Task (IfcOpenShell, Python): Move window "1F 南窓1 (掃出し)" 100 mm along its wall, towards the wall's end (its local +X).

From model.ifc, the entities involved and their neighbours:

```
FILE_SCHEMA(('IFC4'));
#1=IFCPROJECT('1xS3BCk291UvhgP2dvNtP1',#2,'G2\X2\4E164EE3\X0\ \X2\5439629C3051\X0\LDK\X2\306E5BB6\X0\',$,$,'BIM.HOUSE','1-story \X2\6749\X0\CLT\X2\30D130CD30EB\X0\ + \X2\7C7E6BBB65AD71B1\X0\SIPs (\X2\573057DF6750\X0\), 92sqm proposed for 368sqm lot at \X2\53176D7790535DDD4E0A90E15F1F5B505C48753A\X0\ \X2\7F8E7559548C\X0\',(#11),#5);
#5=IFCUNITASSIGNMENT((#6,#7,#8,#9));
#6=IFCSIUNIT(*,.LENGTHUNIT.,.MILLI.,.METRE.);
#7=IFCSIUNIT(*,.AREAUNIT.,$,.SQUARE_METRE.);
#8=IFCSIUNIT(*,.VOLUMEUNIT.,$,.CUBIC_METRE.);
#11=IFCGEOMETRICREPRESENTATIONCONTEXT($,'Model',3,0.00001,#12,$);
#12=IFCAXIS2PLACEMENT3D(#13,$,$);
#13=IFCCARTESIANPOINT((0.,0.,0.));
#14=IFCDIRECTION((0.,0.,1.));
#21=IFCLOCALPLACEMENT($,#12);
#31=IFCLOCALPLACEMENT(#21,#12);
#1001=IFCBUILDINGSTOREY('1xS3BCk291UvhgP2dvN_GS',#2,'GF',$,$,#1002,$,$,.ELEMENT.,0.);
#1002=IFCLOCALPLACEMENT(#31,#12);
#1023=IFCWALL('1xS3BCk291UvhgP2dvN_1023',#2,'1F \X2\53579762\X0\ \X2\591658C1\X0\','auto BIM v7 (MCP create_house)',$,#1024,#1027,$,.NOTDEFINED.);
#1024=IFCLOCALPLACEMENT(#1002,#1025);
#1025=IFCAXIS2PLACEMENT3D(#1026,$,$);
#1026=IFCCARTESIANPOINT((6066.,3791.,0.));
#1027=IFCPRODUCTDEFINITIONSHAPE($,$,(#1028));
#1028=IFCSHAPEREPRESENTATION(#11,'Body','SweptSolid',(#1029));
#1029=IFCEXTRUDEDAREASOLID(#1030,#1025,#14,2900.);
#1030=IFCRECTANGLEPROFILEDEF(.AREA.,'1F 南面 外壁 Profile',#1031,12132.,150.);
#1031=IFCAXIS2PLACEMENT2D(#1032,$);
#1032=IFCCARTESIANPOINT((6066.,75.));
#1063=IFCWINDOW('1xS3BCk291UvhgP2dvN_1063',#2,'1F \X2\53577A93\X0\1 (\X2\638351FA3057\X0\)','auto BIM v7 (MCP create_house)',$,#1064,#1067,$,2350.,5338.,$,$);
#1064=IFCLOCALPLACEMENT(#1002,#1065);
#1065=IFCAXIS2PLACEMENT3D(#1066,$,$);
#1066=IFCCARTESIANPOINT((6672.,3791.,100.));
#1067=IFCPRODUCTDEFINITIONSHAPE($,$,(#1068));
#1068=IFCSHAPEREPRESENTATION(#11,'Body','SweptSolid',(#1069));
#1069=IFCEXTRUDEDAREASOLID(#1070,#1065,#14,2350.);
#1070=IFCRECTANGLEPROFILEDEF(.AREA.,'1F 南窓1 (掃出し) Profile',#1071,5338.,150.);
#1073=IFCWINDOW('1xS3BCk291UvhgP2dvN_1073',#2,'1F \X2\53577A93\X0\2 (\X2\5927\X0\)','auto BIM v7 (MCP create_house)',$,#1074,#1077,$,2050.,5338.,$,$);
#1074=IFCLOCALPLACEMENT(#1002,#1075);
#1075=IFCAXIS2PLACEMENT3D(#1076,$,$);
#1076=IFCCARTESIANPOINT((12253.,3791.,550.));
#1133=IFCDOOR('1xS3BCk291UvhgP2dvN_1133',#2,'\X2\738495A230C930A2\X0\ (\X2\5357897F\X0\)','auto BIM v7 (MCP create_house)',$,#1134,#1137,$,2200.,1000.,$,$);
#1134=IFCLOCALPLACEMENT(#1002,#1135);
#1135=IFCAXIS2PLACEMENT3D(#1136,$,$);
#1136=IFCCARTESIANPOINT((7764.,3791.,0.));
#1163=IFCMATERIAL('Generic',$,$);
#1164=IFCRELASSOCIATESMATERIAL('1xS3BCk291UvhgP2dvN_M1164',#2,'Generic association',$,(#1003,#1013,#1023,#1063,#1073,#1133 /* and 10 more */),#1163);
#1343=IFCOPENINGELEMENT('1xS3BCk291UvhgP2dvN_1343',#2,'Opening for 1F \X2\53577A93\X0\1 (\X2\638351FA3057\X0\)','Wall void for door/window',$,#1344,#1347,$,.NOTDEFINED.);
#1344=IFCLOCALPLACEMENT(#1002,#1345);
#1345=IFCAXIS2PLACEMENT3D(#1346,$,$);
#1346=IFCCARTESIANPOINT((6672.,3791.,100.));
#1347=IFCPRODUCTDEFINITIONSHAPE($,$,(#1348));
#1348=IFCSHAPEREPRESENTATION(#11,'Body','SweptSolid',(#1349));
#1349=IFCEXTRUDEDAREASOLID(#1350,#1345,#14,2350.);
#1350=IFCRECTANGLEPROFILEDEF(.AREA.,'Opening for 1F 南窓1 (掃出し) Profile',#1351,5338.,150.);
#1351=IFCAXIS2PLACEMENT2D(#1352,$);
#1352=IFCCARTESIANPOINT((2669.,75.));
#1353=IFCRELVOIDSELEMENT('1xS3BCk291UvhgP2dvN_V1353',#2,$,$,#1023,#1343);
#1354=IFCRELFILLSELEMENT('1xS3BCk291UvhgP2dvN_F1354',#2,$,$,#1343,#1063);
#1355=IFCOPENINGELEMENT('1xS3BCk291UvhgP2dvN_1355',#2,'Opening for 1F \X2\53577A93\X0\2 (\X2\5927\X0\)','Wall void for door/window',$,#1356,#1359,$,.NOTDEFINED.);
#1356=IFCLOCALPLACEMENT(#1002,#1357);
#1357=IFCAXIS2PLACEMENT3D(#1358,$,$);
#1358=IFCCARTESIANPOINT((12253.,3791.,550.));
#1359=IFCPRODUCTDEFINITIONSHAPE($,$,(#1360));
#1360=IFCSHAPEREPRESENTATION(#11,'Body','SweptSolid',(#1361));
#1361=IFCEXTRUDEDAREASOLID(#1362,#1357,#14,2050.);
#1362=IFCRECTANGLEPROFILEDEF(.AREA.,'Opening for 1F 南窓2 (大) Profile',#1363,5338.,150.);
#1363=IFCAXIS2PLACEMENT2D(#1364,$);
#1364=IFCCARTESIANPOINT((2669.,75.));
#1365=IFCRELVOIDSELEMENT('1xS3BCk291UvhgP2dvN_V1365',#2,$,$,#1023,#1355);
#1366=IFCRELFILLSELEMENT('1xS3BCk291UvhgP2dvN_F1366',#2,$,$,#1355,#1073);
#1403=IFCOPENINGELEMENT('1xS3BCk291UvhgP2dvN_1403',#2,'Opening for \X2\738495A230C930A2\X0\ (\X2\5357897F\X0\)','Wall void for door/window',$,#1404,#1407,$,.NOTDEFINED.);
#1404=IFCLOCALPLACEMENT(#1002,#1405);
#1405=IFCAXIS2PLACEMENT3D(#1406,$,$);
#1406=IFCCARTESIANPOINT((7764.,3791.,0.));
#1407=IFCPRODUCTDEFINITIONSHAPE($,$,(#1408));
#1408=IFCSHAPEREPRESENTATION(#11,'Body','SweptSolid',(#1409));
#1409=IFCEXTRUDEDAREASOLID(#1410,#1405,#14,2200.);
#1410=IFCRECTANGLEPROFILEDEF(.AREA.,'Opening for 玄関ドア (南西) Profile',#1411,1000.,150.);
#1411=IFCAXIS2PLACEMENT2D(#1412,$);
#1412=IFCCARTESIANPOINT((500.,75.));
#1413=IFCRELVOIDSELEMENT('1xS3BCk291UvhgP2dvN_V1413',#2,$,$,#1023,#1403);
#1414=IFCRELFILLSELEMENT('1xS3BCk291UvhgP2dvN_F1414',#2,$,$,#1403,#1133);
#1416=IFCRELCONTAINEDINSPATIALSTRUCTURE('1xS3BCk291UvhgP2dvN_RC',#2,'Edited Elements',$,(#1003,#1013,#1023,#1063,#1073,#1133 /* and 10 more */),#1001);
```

```python
import ifcopenshell
import ifcopenshell.api.geometry
import ifcopenshell.util.placement
import ifcopenshell.util.unit

model = ifcopenshell.open("model.ifc")
unit_scale = ifcopenshell.util.unit.calculate_unit_scale(model)

window = model.by_id(1063)
opening = window.FillsVoids[0].RelatingOpeningElement
wall = opening.VoidsElements[0].RelatingBuildingElement

wall_matrix = ifcopenshell.util.placement.get_local_placement(wall.ObjectPlacement)
shift = wall_matrix[:3, 0] * 0.1 / unit_scale
before = ifcopenshell.util.placement.get_local_placement(window.ObjectPlacement)[:3, 3].copy()

# The window is not placed relative to its opening, so move both.
for product in (opening, window):
    matrix = ifcopenshell.util.placement.get_local_placement(product.ObjectPlacement)
    matrix[:3, 3] += shift
    ifcopenshell.api.geometry.edit_object_placement(model, product=product, matrix=matrix, is_si=False)

after = ifcopenshell.util.placement.get_local_placement(window.ObjectPlacement)[:3, 3]
print("window moved by", (after - before).round(3) + 0.0)

model.write("model-out.ifc")
```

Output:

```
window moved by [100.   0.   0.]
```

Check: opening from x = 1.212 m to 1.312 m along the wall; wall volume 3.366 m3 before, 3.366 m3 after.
